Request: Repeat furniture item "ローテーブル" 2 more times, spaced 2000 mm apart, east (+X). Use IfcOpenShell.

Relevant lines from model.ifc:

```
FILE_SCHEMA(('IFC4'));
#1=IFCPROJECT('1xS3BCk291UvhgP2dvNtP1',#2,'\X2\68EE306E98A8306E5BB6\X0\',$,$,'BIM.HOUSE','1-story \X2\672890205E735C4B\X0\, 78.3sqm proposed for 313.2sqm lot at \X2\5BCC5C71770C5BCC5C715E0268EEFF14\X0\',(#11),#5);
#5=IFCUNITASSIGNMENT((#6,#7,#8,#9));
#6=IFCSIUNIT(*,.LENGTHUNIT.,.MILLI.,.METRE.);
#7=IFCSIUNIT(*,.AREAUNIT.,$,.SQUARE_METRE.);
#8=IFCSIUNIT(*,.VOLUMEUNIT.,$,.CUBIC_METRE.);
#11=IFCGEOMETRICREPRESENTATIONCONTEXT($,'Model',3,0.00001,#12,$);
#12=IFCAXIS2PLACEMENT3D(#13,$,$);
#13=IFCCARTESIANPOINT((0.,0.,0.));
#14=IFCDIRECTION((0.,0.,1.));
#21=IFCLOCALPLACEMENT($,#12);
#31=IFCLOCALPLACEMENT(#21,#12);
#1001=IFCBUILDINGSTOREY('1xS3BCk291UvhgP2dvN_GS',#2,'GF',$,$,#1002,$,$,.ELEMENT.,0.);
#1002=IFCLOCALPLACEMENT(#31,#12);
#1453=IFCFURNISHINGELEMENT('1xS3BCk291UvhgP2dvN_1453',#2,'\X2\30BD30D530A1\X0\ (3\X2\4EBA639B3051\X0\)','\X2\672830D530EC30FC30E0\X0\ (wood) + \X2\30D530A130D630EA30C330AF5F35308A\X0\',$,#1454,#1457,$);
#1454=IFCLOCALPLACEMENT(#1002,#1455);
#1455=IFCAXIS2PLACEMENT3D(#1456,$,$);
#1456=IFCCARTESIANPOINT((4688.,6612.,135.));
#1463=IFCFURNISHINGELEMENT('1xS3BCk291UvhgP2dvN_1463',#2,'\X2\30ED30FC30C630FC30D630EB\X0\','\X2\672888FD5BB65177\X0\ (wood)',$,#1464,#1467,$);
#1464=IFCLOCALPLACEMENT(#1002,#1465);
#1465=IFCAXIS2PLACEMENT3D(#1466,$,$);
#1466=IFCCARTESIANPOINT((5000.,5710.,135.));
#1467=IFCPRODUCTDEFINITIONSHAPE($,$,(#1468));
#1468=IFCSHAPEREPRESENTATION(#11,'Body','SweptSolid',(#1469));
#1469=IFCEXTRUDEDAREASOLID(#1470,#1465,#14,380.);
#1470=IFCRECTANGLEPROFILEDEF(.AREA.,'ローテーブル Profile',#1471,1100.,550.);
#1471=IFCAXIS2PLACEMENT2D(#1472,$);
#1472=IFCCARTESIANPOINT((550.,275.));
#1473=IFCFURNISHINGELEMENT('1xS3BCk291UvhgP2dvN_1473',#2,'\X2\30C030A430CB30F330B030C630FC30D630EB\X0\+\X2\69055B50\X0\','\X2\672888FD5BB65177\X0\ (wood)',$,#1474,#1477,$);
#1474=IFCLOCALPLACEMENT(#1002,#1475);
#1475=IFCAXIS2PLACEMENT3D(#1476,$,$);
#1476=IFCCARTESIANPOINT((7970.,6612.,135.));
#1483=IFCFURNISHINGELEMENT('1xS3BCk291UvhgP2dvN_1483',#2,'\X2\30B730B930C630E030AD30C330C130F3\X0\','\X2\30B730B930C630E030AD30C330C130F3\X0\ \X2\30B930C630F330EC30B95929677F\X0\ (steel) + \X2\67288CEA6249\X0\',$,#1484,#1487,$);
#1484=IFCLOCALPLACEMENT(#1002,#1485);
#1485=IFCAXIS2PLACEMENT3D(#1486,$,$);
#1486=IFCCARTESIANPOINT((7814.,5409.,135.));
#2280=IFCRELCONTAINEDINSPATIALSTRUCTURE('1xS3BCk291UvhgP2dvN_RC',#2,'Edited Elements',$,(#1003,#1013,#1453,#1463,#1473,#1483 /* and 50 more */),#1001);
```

```python
import numpy as np
import ifcopenshell
import ifcopenshell.api.geometry
import ifcopenshell.api.root
import ifcopenshell.util.element
import ifcopenshell.util.placement

model = ifcopenshell.open("model.ifc")


def reuse_history(source, copy):
    """copy_class also copies each property set's owner history, people and application; keep the originals."""
    for rel in copy.IsDefinedBy:
        if rel.is_a("IfcRelDefinesByProperties") and (history := rel.RelatingPropertyDefinition.OwnerHistory):
            rel.RelatingPropertyDefinition.OwnerHistory = source.OwnerHistory
            ifcopenshell.util.element.remove_deep2(model, history)


source = model.by_guid("1xS3BCk291UvhgP2dvN_1463")
base = ifcopenshell.util.placement.get_local_placement(source.ObjectPlacement)
step = np.array([1.0, 0.0, 0.0]) * 2000.0

for i in range(1, 3):
    copy = ifcopenshell.api.root.copy_class(model, product=source)
    copy.Representation = ifcopenshell.util.element.copy_deep(
        model, source.Representation, exclude=["IfcGeometricRepresentationContext", "IfcRepresentationMap"]
    )
    reuse_history(source, copy)
    matrix = base.copy()
    matrix[:3, 3] += i * step
    print("added at", matrix[:3, 3].round(3) + 0.0)
    ifcopenshell.api.geometry.edit_object_placement(model, product=copy, matrix=matrix, is_si=False)

model.write("model_edited.ifc")
```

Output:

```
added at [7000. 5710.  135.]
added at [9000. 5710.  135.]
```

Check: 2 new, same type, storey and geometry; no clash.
